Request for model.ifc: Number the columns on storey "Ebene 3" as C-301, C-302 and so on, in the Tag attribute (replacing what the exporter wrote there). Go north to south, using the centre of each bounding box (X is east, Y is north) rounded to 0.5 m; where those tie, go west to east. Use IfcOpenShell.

First a look at what the model holds.

```python
import ifcopenshell
import ifcopenshell.util.element
import ifcopenshell.util.placement

model = ifcopenshell.open("model.ifc")
print(model.schema)
storey = next(s for s in model.by_type("IfcBuildingStorey") if s.Name == "Ebene 3")
columns = [e for e in ifcopenshell.util.element.get_decomposition(storey) if e.is_a("IfcColumn")]
for e in sorted(columns, key=lambda e: e.id()):
    origin = ifcopenshell.util.placement.get_local_placement(e.ObjectPlacement)[:3, 3]
    print(e.id(), e.Tag, e.Name, origin.round(2) + 0.0, sep=" | ")
```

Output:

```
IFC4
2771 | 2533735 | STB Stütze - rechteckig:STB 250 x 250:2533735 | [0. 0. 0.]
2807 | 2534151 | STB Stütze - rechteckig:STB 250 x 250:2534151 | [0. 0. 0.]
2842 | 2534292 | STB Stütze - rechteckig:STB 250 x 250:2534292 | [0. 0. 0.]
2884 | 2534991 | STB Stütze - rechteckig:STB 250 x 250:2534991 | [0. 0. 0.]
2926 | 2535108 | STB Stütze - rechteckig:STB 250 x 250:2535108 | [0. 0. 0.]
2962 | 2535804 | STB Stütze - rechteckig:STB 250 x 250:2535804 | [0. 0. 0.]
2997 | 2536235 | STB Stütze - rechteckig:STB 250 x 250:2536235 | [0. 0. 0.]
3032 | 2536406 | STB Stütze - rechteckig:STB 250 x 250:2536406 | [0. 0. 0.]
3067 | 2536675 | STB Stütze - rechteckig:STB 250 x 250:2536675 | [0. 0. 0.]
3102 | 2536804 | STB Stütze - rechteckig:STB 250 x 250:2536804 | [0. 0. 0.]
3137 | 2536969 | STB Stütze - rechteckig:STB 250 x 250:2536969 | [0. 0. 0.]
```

```python
import ifcopenshell
import ifcopenshell.geom
import ifcopenshell.util.element
import ifcopenshell.util.shape

model = ifcopenshell.open("model.ifc")
settings = ifcopenshell.geom.settings()
settings.set("use-world-coords", True)


def centre(element):
    shape = ifcopenshell.geom.create_shape(settings, element)
    return ifcopenshell.util.shape.get_bbox_centroid(shape.geometry)


storey = next(s for s in model.by_type("IfcBuildingStorey") if s.Name == "Ebene 3")
columns = [e for e in ifcopenshell.util.element.get_decomposition(storey) if e.is_a("IfcColumn")]

# Insertion points can sit at a corner or the storey origin, so sort by the geometry (in metres).
centres = {e: centre(e) for e in columns}
columns.sort(key=lambda e: (-round(centres[e][1] / 0.5), centres[e][0]))

for i, e in enumerate(columns, start=1):
    number = f"C-3{i:02d}"
    e.Tag = number
    print(e.id(), number)

model.write("model-out.ifc")
```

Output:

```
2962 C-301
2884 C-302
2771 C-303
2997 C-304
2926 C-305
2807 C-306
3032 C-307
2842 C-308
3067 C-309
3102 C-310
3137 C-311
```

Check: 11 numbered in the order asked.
